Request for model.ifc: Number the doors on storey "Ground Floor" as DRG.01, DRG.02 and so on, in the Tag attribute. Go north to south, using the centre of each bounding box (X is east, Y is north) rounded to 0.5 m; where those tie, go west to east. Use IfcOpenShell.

First a look at what the model holds.

```python
import ifcopenshell
import ifcopenshell.util.element
import ifcopenshell.util.placement

model = ifcopenshell.open("model.ifc")
print(model.schema)
storey = next(s for s in model.by_type("IfcBuildingStorey") if s.Name == "Ground Floor")
doors = [e for e in ifcopenshell.util.element.get_decomposition(storey) if e.is_a("IfcDoor")]
for e in sorted(doors, key=lambda e: e.id()):
    origin = ifcopenshell.util.placement.get_local_placement(e.ObjectPlacement)[:3, 3]
    print(e.id(), e.Tag, e.Name, origin.round(2) + 0.0, sep=" | ")
```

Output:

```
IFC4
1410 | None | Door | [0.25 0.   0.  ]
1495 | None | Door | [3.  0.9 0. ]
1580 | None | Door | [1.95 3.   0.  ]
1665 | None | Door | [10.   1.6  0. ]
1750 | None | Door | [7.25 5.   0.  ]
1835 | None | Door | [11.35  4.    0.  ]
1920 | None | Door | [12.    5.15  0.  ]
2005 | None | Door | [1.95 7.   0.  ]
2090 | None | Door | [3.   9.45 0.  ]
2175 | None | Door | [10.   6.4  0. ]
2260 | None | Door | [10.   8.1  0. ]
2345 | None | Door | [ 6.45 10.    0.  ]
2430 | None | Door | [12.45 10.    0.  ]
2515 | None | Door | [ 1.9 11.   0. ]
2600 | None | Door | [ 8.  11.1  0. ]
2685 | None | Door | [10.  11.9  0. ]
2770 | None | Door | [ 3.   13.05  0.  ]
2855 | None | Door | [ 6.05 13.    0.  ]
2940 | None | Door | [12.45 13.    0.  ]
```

```python
import ifcopenshell
import ifcopenshell.geom
import ifcopenshell.util.element
import ifcopenshell.util.shape

model = ifcopenshell.open("model.ifc")
settings = ifcopenshell.geom.settings()
settings.set("use-world-coords", True)


def centre(element):
    shape = ifcopenshell.geom.create_shape(settings, element)
    return ifcopenshell.util.shape.get_bbox_centroid(shape.geometry)


storey = next(s for s in model.by_type("IfcBuildingStorey") if s.Name == "Ground Floor")
doors = [e for e in ifcopenshell.util.element.get_decomposition(storey) if e.is_a("IfcDoor")]

# Insertion points can sit at a corner or the storey origin, so sort by the geometry (in metres).
centres = {e: centre(e) for e in doors}
doors.sort(key=lambda e: (-round(centres[e][1] / 0.5), centres[e][0]))

for i, e in enumerate(doors, start=1):
    number = f"DRG.{i:02d}"
    e.Tag = number
    print(e.id(), number)

model.write("model_edited.ifc")
```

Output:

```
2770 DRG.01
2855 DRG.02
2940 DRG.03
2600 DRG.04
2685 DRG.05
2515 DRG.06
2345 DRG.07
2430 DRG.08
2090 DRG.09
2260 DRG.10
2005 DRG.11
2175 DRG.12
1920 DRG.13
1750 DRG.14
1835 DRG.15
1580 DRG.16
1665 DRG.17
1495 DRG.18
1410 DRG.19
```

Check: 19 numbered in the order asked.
